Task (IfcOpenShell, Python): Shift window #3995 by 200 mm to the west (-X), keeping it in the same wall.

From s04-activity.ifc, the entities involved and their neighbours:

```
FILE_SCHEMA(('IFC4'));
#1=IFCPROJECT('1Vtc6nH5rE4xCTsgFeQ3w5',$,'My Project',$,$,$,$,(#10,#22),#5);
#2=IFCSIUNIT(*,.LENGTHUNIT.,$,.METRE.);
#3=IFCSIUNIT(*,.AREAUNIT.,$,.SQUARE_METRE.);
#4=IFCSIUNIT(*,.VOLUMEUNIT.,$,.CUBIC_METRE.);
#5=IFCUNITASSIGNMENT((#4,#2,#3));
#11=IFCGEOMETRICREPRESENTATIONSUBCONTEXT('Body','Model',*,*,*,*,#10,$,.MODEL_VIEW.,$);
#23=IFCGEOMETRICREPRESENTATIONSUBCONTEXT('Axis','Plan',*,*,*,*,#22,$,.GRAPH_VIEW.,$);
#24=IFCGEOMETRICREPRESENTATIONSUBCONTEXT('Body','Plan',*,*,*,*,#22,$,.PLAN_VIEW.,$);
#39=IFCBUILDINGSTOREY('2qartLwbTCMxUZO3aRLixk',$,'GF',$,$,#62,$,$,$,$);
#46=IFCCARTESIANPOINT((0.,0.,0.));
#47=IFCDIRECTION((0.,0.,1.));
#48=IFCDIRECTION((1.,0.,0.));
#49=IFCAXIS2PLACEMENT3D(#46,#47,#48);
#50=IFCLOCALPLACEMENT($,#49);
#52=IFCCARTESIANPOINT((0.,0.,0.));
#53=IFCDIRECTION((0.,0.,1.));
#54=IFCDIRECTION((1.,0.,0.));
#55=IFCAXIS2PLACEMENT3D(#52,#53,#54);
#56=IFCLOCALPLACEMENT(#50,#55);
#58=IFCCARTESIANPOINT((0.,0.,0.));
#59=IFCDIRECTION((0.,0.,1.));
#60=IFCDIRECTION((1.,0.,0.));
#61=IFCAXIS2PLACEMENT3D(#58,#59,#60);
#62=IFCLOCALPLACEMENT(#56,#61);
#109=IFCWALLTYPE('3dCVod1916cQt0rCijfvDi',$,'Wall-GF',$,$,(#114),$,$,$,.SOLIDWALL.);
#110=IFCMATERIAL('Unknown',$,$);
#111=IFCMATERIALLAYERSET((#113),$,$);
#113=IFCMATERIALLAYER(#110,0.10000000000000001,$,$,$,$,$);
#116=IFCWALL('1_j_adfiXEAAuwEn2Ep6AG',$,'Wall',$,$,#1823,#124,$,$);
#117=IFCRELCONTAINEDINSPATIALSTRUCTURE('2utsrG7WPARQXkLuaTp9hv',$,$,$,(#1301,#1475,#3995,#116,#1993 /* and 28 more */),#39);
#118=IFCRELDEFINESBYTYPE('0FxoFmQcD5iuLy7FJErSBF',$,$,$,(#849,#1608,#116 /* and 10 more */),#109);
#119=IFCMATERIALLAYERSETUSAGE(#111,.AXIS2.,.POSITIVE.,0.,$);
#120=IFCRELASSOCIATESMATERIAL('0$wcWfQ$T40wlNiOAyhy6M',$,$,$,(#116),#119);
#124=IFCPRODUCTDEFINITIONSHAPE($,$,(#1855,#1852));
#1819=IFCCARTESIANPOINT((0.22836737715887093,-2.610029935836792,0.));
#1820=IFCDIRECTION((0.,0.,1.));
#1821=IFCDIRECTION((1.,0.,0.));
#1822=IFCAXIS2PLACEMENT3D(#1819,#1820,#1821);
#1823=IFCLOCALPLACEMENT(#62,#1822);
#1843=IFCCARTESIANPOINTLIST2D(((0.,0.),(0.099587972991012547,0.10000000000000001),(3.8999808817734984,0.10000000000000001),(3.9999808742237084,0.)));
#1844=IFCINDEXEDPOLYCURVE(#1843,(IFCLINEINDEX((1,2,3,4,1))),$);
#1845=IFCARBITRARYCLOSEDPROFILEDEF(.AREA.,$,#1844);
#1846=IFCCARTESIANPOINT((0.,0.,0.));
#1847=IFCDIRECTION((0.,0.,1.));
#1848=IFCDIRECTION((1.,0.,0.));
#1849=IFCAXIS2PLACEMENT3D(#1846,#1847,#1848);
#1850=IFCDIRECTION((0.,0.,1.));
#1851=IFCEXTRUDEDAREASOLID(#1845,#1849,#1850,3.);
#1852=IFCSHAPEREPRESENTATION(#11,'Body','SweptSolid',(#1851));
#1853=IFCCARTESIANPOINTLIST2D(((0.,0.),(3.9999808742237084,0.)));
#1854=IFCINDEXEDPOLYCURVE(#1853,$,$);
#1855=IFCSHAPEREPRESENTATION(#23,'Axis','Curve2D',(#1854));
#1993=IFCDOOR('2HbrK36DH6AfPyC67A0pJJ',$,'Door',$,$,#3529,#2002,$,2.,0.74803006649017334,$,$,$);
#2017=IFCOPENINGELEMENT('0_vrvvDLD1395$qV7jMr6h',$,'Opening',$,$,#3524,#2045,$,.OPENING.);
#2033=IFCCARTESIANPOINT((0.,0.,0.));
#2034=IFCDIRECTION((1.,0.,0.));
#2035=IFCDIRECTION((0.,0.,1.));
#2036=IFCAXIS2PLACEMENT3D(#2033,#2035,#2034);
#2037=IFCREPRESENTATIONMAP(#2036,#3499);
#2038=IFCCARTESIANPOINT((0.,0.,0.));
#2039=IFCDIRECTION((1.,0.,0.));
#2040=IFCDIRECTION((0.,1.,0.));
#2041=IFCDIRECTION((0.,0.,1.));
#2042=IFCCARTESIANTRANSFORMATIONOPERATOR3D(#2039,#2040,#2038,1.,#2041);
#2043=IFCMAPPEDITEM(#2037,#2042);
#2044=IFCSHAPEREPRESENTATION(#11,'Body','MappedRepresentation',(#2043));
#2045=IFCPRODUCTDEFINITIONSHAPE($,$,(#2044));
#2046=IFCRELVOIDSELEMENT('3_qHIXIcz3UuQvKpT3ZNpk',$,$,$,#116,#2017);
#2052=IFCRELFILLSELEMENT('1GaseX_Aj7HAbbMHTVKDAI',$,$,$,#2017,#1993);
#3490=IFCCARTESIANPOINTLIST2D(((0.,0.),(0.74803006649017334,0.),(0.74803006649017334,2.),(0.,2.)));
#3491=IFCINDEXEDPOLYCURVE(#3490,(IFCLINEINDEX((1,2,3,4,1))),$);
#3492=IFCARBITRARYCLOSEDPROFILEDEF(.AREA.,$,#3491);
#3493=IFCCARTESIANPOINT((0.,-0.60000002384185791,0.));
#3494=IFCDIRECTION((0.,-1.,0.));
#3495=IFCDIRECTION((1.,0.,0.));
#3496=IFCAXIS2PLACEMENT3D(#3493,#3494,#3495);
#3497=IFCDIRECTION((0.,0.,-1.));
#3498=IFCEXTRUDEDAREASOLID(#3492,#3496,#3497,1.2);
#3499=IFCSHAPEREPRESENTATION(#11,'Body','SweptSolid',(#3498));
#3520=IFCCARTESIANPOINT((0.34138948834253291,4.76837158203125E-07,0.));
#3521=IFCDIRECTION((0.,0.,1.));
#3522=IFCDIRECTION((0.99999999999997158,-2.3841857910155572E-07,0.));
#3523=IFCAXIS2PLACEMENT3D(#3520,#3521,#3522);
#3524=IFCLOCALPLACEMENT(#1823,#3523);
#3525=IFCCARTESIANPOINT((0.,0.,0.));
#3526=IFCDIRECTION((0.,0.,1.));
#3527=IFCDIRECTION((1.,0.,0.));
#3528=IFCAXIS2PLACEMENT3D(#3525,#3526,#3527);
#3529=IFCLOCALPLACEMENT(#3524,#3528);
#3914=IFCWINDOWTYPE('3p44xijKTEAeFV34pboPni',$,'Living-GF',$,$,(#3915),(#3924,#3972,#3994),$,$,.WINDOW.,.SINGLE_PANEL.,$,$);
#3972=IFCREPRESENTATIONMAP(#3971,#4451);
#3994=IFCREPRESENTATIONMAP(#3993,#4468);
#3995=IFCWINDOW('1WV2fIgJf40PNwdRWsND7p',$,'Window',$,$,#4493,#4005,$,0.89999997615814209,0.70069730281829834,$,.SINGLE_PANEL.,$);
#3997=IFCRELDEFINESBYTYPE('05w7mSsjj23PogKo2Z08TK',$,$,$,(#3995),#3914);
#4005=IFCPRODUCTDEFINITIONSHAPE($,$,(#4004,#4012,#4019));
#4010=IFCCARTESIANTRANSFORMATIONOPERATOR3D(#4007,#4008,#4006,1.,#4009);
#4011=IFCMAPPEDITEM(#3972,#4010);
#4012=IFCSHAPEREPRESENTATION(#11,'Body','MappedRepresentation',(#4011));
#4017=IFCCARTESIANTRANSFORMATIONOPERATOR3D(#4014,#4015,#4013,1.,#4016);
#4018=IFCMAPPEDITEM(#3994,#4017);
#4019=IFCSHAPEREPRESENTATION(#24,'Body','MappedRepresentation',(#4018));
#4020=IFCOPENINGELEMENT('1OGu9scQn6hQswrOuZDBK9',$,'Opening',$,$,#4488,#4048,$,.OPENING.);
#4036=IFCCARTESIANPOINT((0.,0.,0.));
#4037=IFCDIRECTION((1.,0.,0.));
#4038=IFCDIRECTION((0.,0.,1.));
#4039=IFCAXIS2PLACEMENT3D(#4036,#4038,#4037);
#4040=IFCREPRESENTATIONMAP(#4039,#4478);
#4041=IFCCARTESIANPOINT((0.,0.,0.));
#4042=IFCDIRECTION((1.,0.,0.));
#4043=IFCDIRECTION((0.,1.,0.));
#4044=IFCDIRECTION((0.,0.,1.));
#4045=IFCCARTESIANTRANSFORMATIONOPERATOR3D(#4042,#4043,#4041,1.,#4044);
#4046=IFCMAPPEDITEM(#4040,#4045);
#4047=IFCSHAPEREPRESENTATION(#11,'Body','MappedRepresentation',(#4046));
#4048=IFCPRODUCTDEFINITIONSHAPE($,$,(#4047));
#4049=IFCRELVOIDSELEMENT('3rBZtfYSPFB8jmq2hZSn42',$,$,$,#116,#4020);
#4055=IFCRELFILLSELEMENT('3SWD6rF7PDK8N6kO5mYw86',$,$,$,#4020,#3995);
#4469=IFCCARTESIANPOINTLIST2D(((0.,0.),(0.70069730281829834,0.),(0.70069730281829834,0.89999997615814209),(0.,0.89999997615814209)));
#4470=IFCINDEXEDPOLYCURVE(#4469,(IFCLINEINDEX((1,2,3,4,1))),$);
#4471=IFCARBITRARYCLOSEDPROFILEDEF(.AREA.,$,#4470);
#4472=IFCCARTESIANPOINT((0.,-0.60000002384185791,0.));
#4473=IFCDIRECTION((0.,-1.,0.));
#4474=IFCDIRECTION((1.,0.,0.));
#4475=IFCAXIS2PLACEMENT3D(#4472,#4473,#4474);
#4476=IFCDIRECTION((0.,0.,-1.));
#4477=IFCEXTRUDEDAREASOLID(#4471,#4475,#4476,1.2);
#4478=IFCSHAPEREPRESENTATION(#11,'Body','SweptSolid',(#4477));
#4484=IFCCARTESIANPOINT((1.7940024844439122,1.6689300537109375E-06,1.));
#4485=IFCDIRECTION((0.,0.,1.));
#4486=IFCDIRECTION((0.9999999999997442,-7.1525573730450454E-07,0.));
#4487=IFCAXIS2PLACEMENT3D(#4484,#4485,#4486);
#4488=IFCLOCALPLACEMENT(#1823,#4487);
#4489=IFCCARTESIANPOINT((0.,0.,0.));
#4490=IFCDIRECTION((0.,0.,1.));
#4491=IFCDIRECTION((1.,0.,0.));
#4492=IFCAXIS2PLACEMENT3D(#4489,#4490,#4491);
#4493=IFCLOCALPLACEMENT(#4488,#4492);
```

```python
import ifcopenshell
import ifcopenshell.api.geometry
import ifcopenshell.util.placement
import ifcopenshell.util.unit

model = ifcopenshell.open("s04-activity.ifc")
unit_scale = ifcopenshell.util.unit.calculate_unit_scale(model)

window = model.by_guid("1WV2fIgJf40PNwdRWsND7p")
opening = window.FillsVoids[0].RelatingOpeningElement
wall = opening.VoidsElements[0].RelatingBuildingElement

wall_matrix = ifcopenshell.util.placement.get_local_placement(wall.ObjectPlacement)
shift = wall_matrix[:3, 0] * -0.2 / unit_scale
before = ifcopenshell.util.placement.get_local_placement(window.ObjectPlacement)[:3, 3].copy()

# The window is placed relative to its opening, so it follows when the opening moves.
matrix = ifcopenshell.util.placement.get_local_placement(opening.ObjectPlacement)
matrix[:3, 3] += shift
ifcopenshell.api.geometry.edit_object_placement(
    model, product=opening, matrix=matrix, is_si=False, should_transform_children=True
)

after = ifcopenshell.util.placement.get_local_placement(window.ObjectPlacement)[:3, 3]
print("window moved by", (after - before).round(3) + 0.0)

model.write("s04-activity_rev.ifc")
```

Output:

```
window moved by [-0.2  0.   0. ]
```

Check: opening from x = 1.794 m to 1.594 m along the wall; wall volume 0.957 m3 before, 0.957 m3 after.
